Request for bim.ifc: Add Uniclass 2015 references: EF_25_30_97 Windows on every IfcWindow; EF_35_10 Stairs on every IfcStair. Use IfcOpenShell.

First a look at what the model holds.

```python
import ifcopenshell

model = ifcopenshell.open("bim.ifc")
print(model.schema)
print("classifications:", [c.Name for c in model.by_type("IfcClassification")])
for ifc_class in ("IfcDoor", "IfcRoof", "IfcStair", "IfcWall", "IfcWindow"):
    print(ifc_class, len(model.by_type(ifc_class)))
```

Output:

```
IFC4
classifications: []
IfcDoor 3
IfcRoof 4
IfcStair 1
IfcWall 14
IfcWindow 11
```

```python
import ifcopenshell
import ifcopenshell.api.classification

model = ifcopenshell.open("bim.ifc")

system = ifcopenshell.api.classification.add_classification(model, classification="Uniclass 2015")

codes = {
    "IfcWindow": ("EF_25_30_97", "Windows"),
    "IfcStair": ("EF_35_10", "Stairs"),
}
for ifc_class, (code, name) in codes.items():
    products = model.by_type(ifc_class)
    ifcopenshell.api.classification.add_reference(
        model, products=products, classification=system, identification=code, name=name
    )
    print(code, len(products))

model.write("bim_v2.ifc")
```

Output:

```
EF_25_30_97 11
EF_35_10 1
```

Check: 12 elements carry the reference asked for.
